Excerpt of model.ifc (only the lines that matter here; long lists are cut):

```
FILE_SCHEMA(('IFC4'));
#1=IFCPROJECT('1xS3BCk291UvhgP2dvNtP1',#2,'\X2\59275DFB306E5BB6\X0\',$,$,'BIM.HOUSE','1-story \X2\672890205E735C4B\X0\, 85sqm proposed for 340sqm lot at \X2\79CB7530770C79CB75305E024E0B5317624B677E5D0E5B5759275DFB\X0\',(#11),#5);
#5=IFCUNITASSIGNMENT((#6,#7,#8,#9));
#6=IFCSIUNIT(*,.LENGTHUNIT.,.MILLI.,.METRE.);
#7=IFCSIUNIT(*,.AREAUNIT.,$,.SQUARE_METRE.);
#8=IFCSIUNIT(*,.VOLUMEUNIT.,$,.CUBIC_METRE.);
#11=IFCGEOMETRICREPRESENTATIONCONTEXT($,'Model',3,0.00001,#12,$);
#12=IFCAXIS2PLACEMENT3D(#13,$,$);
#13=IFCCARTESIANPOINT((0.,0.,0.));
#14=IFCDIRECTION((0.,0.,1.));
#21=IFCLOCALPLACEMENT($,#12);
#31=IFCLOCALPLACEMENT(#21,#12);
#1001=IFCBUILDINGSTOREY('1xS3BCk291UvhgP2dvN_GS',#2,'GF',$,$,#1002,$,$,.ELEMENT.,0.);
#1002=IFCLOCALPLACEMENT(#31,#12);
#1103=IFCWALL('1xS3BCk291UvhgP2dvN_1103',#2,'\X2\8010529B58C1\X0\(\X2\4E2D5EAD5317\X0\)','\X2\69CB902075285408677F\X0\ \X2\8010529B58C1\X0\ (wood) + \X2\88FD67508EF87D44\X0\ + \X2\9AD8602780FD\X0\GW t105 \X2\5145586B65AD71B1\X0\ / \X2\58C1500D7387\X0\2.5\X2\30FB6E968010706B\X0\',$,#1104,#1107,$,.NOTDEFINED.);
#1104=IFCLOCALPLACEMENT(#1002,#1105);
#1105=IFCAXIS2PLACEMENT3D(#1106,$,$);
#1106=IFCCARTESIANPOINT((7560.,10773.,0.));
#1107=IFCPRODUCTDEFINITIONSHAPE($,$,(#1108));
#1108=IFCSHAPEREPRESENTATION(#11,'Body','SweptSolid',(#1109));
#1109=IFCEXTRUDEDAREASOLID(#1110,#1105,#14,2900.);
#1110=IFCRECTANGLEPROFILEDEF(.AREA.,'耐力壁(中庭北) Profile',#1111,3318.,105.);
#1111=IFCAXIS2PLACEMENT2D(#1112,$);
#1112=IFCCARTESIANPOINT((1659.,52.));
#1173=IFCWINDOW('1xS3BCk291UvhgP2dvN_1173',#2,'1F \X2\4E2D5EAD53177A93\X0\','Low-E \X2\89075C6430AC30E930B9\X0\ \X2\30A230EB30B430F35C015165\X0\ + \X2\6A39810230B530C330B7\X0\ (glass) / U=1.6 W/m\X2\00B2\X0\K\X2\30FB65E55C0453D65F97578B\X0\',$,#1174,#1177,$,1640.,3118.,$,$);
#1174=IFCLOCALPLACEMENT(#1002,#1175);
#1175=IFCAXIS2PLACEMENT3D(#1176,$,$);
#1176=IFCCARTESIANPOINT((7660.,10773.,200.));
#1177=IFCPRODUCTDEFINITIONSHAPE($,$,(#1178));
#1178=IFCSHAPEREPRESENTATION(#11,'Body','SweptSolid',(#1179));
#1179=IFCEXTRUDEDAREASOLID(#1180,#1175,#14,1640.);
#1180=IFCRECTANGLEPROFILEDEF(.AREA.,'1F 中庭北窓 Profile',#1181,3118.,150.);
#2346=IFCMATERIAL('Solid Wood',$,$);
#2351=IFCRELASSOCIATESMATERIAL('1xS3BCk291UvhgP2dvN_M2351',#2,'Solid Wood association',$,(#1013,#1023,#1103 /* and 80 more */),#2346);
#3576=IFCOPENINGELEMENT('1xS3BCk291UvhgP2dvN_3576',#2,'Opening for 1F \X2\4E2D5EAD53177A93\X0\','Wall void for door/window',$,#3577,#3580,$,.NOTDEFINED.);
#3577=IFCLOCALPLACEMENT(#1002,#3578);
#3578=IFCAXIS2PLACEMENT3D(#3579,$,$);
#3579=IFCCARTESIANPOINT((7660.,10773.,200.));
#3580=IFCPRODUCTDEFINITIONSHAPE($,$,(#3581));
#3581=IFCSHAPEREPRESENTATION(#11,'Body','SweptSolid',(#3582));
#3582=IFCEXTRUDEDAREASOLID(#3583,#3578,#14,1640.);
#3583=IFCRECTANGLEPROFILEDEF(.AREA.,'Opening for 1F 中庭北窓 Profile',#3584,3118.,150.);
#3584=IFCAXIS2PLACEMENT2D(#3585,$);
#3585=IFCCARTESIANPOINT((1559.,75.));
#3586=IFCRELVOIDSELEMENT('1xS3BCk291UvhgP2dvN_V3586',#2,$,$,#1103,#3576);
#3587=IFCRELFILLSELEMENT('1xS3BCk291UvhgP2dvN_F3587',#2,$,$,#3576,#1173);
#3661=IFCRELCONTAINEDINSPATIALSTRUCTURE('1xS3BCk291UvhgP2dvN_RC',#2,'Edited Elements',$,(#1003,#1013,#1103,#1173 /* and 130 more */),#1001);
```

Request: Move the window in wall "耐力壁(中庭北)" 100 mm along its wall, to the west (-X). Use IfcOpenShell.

```python
import ifcopenshell
import ifcopenshell.api.geometry
import ifcopenshell.util.placement
import ifcopenshell.util.unit

model = ifcopenshell.open("model.ifc")
unit_scale = ifcopenshell.util.unit.calculate_unit_scale(model)

window = model.by_guid("1xS3BCk291UvhgP2dvN_1173")
opening = window.FillsVoids[0].RelatingOpeningElement
wall = opening.VoidsElements[0].RelatingBuildingElement

wall_matrix = ifcopenshell.util.placement.get_local_placement(wall.ObjectPlacement)
shift = wall_matrix[:3, 0] * -0.1 / unit_scale
before = ifcopenshell.util.placement.get_local_placement(window.ObjectPlacement)[:3, 3].copy()

# The window is not placed relative to its opening, so move both.
for product in (opening, window):
    matrix = ifcopenshell.util.placement.get_local_placement(product.ObjectPlacement)
    matrix[:3, 3] += shift
    ifcopenshell.api.geometry.edit_object_placement(model, product=product, matrix=matrix, is_si=False)

after = ifcopenshell.util.placement.get_local_placement(window.ObjectPlacement)[:3, 3]
print("window moved by", (after - before).round(3) + 0.0)

model.write("model-out.ifc")
```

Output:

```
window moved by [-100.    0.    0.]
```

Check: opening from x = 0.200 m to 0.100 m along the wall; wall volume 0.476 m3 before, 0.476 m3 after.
